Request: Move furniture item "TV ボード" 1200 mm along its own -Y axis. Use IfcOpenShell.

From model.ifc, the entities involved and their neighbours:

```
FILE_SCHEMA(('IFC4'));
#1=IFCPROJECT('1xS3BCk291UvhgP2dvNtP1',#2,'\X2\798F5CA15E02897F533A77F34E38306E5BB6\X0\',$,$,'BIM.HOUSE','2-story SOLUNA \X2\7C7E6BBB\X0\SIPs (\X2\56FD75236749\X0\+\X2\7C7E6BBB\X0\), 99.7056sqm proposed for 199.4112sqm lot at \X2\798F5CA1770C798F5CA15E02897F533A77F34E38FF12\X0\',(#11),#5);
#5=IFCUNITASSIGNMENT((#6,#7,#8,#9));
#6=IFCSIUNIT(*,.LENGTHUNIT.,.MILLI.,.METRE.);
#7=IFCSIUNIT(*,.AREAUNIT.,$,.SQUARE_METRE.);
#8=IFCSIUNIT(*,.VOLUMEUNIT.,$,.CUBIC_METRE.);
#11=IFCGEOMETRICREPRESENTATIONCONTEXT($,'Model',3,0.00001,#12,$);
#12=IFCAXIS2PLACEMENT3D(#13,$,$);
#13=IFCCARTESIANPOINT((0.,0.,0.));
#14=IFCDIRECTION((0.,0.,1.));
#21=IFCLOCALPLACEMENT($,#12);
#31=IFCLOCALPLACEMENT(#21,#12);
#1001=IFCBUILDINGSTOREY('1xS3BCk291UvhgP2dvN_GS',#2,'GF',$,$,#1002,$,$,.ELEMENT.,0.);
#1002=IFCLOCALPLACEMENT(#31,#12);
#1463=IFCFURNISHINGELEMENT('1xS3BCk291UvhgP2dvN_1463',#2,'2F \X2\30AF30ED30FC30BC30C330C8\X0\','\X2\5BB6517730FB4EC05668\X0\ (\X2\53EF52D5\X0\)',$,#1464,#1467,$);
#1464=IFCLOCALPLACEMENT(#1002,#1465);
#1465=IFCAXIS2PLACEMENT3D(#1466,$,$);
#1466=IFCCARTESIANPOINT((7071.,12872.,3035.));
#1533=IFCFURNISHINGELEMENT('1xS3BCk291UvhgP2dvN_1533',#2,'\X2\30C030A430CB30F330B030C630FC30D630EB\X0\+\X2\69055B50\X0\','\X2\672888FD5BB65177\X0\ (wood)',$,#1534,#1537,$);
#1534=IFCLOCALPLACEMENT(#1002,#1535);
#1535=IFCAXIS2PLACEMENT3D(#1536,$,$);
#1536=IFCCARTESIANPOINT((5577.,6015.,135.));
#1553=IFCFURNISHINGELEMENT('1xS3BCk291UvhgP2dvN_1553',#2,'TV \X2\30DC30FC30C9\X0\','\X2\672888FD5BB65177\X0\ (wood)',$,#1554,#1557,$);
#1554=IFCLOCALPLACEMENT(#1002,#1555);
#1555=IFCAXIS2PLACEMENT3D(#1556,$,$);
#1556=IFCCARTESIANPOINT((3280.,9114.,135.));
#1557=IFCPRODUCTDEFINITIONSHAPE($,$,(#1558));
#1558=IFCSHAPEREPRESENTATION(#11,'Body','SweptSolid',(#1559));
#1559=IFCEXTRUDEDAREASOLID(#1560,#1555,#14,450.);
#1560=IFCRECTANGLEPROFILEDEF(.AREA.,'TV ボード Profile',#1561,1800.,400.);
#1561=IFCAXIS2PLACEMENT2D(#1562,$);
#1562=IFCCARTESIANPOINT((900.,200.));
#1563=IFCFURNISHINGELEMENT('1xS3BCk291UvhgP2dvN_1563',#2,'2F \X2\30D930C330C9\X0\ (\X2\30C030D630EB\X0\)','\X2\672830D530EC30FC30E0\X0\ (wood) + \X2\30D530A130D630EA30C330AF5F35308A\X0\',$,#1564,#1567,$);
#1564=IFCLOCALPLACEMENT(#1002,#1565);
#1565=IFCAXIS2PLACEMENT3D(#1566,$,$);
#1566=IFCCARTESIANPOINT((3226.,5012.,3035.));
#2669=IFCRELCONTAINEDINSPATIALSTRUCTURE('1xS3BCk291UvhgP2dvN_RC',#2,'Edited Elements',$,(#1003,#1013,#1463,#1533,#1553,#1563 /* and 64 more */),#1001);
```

```python
import ifcopenshell
import ifcopenshell.api.geometry
import ifcopenshell.util.placement

model = ifcopenshell.open("model.ifc")

item = model.by_guid("1xS3BCk291UvhgP2dvN_1553")
matrix = ifcopenshell.util.placement.get_local_placement(item.ObjectPlacement)
matrix[:3, 3] -= matrix[:3, 1] * 1200.0
ifcopenshell.api.geometry.edit_object_placement(model, product=item, matrix=matrix, is_si=False)

print(ifcopenshell.util.placement.get_local_placement(item.ObjectPlacement).round(3) + 0.0)

model.write("model-out.ifc")
```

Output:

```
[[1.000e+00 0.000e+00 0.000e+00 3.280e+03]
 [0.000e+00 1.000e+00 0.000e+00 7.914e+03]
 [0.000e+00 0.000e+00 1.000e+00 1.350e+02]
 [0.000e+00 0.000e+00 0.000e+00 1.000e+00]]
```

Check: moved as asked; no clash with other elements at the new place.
